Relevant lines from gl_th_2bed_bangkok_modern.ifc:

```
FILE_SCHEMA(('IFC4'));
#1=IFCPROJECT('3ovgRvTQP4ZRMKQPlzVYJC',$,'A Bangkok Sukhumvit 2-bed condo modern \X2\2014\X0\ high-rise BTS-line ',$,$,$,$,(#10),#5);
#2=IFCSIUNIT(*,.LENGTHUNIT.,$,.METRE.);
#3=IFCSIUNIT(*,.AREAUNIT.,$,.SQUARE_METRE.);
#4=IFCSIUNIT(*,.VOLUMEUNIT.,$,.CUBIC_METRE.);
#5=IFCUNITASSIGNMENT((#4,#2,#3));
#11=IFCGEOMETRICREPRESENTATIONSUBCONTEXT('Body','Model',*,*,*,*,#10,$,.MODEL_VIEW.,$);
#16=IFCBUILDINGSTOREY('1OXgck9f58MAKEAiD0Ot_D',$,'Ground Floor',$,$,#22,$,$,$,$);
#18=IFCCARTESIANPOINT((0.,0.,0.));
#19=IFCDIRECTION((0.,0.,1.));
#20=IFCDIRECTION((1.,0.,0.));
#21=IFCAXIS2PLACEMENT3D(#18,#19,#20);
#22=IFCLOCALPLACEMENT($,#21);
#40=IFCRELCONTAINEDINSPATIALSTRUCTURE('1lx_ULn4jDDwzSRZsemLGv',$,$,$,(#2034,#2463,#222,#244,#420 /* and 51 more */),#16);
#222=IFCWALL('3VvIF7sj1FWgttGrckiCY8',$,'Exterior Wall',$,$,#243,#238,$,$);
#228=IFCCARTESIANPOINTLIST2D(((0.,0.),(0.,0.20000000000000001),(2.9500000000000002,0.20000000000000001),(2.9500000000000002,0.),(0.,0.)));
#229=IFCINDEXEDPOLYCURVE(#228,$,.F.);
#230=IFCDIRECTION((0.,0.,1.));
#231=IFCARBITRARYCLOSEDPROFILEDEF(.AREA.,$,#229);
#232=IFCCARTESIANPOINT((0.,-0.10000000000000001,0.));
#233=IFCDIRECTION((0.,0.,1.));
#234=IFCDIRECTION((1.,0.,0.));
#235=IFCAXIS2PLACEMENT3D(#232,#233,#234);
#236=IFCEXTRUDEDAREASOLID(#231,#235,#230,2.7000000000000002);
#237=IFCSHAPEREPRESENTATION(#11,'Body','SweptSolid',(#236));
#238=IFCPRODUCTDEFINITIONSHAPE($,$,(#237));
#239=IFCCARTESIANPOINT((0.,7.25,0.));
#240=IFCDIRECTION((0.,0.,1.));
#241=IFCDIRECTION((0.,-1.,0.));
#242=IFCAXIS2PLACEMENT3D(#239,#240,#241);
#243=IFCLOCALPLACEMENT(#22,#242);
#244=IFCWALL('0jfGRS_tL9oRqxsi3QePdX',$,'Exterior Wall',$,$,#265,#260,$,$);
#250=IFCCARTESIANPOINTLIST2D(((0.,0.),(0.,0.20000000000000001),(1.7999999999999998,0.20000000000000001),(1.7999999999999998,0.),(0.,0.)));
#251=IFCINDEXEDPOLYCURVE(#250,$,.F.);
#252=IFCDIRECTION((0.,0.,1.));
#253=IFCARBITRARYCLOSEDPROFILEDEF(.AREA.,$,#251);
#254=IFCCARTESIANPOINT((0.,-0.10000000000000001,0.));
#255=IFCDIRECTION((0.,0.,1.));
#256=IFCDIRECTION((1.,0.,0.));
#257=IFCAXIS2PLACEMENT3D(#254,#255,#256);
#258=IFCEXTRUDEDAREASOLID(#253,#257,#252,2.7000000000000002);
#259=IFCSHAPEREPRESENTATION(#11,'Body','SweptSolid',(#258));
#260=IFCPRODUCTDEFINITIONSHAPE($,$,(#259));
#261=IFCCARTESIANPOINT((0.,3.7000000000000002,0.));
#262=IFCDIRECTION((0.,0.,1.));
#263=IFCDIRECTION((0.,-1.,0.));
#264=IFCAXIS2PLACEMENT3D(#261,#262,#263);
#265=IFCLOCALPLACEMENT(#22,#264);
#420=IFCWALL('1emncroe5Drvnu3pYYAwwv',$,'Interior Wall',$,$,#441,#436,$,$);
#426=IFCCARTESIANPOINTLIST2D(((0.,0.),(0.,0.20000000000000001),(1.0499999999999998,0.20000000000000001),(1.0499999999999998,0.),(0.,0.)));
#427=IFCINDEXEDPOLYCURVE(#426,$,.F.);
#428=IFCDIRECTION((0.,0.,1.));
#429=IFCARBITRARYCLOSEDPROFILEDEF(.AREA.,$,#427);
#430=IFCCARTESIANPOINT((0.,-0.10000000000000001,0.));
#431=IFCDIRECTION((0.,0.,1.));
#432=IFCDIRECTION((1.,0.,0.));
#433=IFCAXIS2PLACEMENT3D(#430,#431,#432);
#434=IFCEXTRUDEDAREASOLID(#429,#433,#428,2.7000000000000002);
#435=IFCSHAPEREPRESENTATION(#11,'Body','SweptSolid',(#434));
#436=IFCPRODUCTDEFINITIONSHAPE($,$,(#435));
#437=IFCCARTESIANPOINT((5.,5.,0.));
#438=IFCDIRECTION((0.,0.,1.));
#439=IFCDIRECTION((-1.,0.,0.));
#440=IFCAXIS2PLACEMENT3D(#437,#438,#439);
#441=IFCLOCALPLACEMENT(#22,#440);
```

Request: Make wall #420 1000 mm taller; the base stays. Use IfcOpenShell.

```python
import ifcopenshell
import ifcopenshell.geom
import ifcopenshell.util.representation
import ifcopenshell.util.shape
import ifcopenshell.util.unit

model = ifcopenshell.open("gl_th_2bed_bangkok_modern.ifc")
unit_scale = ifcopenshell.util.unit.calculate_unit_scale(model)
settings = ifcopenshell.geom.settings()


def volume(element):
    """Net volume in cubic metres, openings subtracted."""
    shape = ifcopenshell.geom.create_shape(settings, element)
    return ifcopenshell.util.shape.get_volume(shape.geometry)


wall = model.by_id(420)
before = volume(wall)

body = ifcopenshell.util.representation.get_representation(wall, "Model", "Body")
solid = body.Items[0]
old_height = solid.Depth
solid.Depth += 1 / unit_scale
after = volume(wall)

print(f"height {old_height:g} -> {solid.Depth:g}, volume {before:.3f} -> {after:.3f} m3")

model.write("gl_th_2bed_bangkok_modern_updated.ifc")
```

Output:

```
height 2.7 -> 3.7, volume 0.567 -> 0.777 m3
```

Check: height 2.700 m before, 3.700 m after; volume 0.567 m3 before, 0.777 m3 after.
